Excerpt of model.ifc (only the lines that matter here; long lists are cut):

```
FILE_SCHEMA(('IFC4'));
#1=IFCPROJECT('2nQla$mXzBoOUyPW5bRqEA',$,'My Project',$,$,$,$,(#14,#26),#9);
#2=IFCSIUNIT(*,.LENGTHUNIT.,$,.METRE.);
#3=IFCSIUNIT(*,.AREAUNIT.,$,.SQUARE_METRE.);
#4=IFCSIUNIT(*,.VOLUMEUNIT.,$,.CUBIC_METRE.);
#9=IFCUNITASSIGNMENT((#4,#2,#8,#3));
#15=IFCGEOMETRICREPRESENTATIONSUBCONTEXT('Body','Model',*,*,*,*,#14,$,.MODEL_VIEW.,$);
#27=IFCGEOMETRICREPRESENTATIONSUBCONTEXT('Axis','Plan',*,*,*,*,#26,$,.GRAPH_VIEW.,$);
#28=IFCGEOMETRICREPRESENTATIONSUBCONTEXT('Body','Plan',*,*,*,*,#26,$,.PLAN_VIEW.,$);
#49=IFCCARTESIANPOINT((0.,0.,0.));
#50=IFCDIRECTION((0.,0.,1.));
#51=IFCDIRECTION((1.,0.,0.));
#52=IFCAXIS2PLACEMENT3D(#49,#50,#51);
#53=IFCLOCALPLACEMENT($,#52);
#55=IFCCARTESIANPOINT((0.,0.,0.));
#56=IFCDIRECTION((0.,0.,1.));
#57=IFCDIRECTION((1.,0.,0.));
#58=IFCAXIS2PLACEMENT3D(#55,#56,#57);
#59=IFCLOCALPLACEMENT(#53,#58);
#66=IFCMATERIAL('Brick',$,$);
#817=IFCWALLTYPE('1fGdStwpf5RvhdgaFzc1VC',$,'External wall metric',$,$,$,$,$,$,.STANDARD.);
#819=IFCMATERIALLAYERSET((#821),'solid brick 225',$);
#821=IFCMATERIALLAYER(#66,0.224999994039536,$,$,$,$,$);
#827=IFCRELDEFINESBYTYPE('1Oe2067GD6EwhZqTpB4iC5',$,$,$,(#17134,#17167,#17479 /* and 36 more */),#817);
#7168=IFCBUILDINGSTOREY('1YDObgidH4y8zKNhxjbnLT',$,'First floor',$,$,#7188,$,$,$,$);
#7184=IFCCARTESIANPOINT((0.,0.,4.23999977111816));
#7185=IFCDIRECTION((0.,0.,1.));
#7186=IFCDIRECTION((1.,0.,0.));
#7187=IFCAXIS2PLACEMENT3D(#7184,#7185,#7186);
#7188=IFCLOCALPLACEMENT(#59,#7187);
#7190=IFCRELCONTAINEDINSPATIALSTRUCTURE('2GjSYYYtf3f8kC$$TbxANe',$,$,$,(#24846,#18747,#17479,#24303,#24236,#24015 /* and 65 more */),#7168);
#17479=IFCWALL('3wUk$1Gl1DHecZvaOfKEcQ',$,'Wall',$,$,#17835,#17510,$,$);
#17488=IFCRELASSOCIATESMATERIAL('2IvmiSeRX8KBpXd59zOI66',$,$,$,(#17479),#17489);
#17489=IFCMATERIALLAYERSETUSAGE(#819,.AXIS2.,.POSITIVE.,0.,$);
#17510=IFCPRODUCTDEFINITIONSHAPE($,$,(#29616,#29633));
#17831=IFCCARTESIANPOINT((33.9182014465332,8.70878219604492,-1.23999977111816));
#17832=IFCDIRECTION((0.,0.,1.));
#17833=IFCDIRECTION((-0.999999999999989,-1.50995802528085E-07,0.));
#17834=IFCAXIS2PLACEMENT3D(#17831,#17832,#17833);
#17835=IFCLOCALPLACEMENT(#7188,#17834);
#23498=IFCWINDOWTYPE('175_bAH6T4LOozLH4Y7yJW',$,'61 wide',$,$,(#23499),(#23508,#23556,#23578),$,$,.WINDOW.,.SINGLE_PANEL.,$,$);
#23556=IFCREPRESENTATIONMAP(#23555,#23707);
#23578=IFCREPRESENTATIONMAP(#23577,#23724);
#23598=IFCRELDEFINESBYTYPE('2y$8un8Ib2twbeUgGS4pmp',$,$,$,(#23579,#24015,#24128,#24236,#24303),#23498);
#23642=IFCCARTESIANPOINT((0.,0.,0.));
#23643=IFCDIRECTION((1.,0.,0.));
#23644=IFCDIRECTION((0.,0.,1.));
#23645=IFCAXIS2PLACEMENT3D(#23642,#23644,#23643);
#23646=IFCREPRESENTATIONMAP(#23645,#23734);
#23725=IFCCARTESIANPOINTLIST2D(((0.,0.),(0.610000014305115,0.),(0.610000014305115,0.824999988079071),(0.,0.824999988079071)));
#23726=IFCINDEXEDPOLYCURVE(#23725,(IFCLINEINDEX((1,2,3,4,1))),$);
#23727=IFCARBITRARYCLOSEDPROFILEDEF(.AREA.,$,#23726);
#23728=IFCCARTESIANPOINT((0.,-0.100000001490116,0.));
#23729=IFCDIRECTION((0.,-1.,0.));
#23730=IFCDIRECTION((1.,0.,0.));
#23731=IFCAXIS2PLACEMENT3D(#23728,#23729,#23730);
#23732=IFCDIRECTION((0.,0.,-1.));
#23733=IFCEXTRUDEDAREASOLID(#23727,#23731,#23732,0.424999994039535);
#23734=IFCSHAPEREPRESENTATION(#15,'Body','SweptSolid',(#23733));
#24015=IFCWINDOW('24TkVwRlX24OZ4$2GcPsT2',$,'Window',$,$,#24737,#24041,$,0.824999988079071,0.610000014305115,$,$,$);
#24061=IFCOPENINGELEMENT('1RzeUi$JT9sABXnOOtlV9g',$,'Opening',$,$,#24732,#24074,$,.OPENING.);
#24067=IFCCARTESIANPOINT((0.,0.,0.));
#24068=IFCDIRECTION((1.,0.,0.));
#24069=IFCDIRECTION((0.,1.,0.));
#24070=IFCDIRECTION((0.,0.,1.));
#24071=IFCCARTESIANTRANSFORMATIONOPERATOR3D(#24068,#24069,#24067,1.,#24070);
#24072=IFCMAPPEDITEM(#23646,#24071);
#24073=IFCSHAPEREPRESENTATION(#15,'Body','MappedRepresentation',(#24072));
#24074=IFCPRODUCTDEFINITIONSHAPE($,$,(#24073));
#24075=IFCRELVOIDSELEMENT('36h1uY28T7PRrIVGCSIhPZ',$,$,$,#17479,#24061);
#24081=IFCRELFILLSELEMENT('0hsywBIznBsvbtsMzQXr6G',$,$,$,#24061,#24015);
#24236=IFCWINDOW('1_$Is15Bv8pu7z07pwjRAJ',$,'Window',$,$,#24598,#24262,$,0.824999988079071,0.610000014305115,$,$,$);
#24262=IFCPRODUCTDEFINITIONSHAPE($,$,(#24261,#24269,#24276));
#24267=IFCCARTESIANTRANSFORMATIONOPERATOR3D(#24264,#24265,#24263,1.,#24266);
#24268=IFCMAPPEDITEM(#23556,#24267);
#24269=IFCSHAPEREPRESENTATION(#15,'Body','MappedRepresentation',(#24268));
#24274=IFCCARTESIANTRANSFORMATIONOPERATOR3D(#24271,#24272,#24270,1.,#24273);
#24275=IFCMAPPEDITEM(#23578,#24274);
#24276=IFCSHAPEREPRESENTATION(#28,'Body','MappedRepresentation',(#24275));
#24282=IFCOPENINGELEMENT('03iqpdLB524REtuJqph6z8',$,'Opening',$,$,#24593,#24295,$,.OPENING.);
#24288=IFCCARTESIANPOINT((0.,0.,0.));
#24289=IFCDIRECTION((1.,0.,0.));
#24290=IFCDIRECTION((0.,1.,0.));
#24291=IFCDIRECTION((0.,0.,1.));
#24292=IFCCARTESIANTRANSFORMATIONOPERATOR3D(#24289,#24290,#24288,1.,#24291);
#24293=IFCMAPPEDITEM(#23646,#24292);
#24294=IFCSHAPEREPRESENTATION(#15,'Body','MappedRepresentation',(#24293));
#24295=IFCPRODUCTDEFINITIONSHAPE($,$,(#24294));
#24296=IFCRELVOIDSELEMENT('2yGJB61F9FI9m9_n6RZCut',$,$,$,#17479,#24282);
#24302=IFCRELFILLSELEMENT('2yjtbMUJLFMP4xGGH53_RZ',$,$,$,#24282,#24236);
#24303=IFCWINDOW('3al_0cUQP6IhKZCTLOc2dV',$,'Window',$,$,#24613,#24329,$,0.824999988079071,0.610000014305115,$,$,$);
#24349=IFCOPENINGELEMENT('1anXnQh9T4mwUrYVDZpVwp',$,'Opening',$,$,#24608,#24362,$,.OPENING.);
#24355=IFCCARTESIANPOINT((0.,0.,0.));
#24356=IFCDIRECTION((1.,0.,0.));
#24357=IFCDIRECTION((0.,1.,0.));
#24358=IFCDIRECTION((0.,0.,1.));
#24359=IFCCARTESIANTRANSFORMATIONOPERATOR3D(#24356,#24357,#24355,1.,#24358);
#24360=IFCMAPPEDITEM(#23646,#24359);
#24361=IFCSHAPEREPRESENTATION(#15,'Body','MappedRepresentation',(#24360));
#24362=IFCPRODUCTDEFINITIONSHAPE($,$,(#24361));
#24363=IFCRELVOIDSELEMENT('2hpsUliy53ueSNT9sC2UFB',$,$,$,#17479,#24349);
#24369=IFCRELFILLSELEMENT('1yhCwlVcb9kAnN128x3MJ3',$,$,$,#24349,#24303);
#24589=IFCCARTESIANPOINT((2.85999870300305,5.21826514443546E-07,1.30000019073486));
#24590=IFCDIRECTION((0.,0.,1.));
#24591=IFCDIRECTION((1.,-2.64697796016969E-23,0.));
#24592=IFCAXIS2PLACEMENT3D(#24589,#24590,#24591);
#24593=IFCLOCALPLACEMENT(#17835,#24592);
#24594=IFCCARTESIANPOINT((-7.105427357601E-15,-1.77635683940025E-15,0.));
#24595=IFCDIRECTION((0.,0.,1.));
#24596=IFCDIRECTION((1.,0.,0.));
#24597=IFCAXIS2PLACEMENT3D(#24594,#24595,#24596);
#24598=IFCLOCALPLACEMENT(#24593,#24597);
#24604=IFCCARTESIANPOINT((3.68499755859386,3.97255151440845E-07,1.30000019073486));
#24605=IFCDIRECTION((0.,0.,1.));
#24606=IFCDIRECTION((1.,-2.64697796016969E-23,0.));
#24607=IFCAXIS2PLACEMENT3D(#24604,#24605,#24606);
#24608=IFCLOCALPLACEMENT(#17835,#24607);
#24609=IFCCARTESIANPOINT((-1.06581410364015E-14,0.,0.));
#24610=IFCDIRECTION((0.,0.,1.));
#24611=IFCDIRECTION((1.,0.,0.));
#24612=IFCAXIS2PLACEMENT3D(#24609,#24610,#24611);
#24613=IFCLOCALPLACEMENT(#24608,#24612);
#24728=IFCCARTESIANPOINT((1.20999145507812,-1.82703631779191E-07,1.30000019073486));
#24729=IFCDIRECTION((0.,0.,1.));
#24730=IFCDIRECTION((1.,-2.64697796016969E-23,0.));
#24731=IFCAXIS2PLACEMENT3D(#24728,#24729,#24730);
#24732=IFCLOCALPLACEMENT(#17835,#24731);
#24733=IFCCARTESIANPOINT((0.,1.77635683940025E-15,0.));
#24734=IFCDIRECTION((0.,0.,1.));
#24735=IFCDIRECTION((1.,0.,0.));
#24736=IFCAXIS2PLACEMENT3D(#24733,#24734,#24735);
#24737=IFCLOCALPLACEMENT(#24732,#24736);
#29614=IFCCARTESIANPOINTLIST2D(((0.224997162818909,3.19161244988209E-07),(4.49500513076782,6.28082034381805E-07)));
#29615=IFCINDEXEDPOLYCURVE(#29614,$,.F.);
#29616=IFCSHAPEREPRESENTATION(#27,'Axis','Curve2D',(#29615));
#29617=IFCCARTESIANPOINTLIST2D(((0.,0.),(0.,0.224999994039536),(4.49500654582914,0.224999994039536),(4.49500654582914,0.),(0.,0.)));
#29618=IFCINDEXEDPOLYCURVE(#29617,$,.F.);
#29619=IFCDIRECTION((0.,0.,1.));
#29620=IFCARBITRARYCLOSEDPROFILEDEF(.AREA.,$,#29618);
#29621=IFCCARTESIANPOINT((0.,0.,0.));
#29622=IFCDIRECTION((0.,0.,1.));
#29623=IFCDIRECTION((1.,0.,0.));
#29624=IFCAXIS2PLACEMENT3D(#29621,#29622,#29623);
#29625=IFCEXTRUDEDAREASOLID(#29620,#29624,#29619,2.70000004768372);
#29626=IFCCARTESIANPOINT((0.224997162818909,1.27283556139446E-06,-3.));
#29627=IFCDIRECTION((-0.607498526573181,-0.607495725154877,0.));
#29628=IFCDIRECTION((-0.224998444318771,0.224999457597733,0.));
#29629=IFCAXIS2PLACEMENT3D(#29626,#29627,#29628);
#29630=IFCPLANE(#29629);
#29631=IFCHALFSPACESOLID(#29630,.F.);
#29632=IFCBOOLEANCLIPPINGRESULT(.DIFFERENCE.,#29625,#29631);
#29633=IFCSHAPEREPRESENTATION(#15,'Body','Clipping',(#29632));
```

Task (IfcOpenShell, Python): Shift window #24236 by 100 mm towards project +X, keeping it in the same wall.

```python
import ifcopenshell
import ifcopenshell.api.geometry
import ifcopenshell.util.placement

model = ifcopenshell.open("model.ifc")

window = model.by_guid("1_$Is15Bv8pu7z07pwjRAJ")
opening = window.FillsVoids[0].RelatingOpeningElement
wall = opening.VoidsElements[0].RelatingBuildingElement

wall_matrix = ifcopenshell.util.placement.get_local_placement(wall.ObjectPlacement)
shift = wall_matrix[:3, 0] * -0.1
before = ifcopenshell.util.placement.get_local_placement(window.ObjectPlacement)[:3, 3].copy()

# The window is placed relative to its opening, so it follows when the opening moves.
matrix = ifcopenshell.util.placement.get_local_placement(opening.ObjectPlacement)
matrix[:3, 3] += shift
ifcopenshell.api.geometry.edit_object_placement(
    model, product=opening, matrix=matrix, is_si=False, should_transform_children=True
)

after = ifcopenshell.util.placement.get_local_placement(window.ObjectPlacement)[:3, 3]
print("window moved by", (after - before).round(3) + 0.0)

model.write("model_rev.ifc")
```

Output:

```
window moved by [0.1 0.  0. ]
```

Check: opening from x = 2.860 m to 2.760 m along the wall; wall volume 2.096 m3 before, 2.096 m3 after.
